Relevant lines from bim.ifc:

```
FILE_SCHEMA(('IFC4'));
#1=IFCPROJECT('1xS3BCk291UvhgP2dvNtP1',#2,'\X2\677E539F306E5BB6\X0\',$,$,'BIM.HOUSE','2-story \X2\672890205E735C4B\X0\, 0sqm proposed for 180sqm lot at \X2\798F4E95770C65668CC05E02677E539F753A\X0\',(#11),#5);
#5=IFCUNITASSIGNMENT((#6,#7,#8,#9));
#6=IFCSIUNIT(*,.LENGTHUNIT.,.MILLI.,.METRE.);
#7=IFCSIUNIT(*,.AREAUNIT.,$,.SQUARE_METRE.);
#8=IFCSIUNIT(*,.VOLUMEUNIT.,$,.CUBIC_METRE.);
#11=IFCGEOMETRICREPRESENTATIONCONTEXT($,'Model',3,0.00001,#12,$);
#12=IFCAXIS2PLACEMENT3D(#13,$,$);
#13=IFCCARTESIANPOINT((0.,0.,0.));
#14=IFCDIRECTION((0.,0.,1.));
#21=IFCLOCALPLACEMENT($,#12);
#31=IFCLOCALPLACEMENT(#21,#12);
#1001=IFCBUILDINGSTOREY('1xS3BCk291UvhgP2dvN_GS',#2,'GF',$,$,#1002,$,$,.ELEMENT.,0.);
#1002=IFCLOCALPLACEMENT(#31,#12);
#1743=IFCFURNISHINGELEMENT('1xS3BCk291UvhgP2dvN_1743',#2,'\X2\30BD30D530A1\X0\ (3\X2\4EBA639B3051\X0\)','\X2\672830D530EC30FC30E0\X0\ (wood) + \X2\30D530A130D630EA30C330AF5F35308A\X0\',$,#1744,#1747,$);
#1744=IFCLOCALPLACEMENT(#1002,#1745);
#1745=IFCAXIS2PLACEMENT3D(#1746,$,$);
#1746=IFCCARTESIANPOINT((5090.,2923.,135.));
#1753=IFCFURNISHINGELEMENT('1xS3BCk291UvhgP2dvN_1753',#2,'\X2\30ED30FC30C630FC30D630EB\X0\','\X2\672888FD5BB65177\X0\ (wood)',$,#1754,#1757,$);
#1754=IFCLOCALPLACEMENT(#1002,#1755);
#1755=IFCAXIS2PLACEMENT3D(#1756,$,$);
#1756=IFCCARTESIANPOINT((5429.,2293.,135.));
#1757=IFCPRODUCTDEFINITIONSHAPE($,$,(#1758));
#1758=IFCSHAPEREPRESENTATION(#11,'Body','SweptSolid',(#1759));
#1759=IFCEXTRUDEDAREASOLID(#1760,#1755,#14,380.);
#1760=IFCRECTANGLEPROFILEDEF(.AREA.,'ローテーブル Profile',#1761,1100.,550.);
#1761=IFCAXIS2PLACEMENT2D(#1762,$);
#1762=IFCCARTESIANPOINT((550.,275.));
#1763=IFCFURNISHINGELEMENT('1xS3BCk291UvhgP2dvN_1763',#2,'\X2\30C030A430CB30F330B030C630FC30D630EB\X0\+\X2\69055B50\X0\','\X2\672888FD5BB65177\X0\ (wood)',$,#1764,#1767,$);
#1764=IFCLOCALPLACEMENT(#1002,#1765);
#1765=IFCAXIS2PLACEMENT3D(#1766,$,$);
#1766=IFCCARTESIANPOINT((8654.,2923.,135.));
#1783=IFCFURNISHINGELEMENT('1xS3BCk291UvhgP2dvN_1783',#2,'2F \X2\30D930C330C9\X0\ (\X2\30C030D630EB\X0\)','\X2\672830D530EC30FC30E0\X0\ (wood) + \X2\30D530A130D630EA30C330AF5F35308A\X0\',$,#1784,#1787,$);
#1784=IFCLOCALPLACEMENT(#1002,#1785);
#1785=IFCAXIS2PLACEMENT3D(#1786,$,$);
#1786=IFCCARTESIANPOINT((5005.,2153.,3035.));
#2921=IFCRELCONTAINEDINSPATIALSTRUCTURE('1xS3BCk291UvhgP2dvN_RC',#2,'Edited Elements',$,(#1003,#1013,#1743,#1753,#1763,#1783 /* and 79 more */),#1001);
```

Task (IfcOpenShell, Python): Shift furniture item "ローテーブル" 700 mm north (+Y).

```python
import ifcopenshell
import ifcopenshell.api.geometry
import ifcopenshell.util.placement

model = ifcopenshell.open("bim.ifc")

item = model.by_id(1753)
matrix = ifcopenshell.util.placement.get_local_placement(item.ObjectPlacement)
matrix[1, 3] += 700.0
ifcopenshell.api.geometry.edit_object_placement(model, product=item, matrix=matrix, is_si=False)

print(ifcopenshell.util.placement.get_local_placement(item.ObjectPlacement).round(3) + 0.0)

model.write("bim-out.ifc")
```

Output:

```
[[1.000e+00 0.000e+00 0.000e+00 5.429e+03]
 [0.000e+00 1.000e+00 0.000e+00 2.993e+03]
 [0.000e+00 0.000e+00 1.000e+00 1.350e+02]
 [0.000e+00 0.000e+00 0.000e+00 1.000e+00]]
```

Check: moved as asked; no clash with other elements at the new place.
